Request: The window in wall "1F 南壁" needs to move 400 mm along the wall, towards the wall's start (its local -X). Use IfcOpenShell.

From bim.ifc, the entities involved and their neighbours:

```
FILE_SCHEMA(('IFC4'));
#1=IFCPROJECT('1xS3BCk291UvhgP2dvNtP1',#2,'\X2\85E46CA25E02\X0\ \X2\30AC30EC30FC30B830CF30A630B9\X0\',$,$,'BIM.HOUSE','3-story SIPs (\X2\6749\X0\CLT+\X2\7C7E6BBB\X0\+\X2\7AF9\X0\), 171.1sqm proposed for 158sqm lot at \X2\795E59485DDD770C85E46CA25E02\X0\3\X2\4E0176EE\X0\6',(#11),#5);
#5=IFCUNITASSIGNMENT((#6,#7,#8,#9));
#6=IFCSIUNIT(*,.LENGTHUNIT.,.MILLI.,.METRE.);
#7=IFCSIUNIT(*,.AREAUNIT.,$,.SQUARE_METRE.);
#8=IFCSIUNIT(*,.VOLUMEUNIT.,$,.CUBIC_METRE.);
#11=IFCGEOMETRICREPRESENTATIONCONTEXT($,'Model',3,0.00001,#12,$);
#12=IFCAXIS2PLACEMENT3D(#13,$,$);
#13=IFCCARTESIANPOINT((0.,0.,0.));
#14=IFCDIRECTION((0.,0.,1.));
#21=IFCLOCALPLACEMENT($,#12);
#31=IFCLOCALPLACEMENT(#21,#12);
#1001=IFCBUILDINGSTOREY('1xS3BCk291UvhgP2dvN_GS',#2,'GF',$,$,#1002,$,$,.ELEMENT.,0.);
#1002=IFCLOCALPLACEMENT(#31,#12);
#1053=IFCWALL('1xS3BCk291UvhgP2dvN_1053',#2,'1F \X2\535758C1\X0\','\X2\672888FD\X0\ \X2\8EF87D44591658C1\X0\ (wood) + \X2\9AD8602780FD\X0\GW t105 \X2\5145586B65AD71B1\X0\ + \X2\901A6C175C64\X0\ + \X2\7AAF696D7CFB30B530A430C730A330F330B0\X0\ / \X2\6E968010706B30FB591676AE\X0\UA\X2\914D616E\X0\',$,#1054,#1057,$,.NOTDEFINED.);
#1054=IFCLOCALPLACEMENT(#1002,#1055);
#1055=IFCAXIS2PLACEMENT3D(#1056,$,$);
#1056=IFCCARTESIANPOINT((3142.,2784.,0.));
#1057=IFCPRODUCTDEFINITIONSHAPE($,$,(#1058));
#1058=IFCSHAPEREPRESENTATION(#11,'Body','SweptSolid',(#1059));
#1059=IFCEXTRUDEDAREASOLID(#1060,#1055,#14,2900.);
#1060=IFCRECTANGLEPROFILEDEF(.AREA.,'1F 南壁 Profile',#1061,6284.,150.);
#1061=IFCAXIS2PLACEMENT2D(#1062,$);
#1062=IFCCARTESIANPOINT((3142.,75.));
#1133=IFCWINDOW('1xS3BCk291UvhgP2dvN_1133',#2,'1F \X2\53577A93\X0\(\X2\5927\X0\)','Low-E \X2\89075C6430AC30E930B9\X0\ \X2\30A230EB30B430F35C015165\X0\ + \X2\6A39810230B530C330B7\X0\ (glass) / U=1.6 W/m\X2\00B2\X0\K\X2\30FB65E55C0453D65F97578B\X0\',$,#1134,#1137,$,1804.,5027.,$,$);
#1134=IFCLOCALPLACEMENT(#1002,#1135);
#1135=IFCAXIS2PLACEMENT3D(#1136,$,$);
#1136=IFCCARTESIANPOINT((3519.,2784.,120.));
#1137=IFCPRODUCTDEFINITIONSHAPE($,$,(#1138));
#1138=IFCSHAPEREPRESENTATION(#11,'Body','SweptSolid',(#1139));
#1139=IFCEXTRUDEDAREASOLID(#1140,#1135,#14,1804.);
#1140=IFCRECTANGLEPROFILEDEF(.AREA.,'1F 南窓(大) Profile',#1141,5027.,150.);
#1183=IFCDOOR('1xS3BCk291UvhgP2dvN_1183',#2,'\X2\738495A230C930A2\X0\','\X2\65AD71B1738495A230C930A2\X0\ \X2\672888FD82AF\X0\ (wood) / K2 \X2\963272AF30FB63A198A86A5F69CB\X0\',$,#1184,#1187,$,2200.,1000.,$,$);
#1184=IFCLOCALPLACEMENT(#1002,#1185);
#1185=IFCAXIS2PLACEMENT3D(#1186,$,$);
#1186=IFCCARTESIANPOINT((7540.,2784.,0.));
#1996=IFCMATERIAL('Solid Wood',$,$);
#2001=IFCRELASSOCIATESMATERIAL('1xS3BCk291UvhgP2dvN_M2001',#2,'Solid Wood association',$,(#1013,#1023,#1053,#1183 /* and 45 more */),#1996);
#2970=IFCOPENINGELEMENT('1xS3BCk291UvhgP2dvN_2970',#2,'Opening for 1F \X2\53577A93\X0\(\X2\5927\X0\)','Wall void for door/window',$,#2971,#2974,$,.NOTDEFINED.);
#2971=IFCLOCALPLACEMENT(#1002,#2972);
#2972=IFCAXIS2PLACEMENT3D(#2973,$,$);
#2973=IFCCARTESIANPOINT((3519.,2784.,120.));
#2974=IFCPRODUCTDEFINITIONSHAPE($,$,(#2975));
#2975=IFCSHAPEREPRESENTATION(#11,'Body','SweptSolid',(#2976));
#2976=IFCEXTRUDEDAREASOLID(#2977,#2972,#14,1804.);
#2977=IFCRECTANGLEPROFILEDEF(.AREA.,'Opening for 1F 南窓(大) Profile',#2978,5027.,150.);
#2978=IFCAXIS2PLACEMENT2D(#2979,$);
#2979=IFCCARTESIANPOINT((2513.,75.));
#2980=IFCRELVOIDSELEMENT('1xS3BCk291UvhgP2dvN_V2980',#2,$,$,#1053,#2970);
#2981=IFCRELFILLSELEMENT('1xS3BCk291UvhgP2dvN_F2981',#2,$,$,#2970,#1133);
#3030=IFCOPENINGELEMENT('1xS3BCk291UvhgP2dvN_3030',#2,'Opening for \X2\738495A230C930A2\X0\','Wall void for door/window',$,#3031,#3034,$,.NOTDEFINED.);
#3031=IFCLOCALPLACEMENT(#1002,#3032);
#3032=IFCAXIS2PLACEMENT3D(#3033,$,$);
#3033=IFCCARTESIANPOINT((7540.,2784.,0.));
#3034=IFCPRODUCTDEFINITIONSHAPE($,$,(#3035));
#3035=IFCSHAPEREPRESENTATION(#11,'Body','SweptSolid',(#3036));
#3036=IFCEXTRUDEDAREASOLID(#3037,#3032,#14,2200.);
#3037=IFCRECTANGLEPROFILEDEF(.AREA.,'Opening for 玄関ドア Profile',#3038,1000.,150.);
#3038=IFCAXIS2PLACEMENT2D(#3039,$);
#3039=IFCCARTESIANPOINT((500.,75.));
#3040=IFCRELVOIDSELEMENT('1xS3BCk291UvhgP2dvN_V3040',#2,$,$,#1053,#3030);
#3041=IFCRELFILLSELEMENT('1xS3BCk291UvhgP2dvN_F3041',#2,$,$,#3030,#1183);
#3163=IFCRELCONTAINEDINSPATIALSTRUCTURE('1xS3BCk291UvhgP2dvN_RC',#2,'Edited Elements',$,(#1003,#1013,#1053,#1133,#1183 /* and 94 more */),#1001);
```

```python
import ifcopenshell
import ifcopenshell.api.geometry
import ifcopenshell.util.placement

model = ifcopenshell.open("bim.ifc")

window = model.by_guid("1xS3BCk291UvhgP2dvN_1133")
opening = window.FillsVoids[0].RelatingOpeningElement
wall = opening.VoidsElements[0].RelatingBuildingElement

wall_matrix = ifcopenshell.util.placement.get_local_placement(wall.ObjectPlacement)
shift = wall_matrix[:3, 0] * -400.0
before = ifcopenshell.util.placement.get_local_placement(window.ObjectPlacement)[:3, 3].copy()

# The window is not placed relative to its opening, so move both.
for product in (opening, window):
    matrix = ifcopenshell.util.placement.get_local_placement(product.ObjectPlacement)
    matrix[:3, 3] += shift
    ifcopenshell.api.geometry.edit_object_placement(model, product=product, matrix=matrix, is_si=False)

after = ifcopenshell.util.placement.get_local_placement(window.ObjectPlacement)[:3, 3]
print("window moved by", (after - before).round(3) + 0.0)

model.write("bim-out.ifc")
```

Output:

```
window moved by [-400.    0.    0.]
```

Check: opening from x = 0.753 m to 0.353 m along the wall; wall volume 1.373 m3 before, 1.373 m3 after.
